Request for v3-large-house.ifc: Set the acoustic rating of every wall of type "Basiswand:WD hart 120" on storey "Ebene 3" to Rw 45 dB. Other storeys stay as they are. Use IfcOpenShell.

First a look at what the model holds.

```python
import ifcopenshell
import ifcopenshell.util.element

model = ifcopenshell.open("v3-large-house.ifc")
print(model.schema)
storey = next(s for s in model.by_type("IfcBuildingStorey") if s.Name == "Ebene 3")
walls = [e for e in ifcopenshell.util.element.get_decomposition(storey) if e.is_a("IfcWall")]
seen = {}
for e in walls:
    element_type = ifcopenshell.util.element.get_type(e)
    key = (element_type.Name if element_type != e and element_type else None, ifcopenshell.util.element.get_pset(e, "Pset_WallCommon", "AcousticRating"))
    seen[key] = seen.get(key, 0) + 1
for (name, value), count in sorted(seen.items(), key=str):
    print(count, "x", name, "|", value)
```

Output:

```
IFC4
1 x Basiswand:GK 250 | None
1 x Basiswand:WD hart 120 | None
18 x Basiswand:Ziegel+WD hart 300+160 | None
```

```python
import ifcopenshell
import ifcopenshell.api.pset
import ifcopenshell.util.element

model = ifcopenshell.open("v3-large-house.ifc")

storey = next(s for s in model.by_type("IfcBuildingStorey") if s.Name == "Ebene 3")
walls = [e for e in ifcopenshell.util.element.get_decomposition(storey) if e.is_a("IfcWall")]

count = 0
for e in walls:
    element_type = ifcopenshell.util.element.get_type(e)
    if element_type in (None, e) or element_type.Name != "Basiswand:WD hart 120":
        continue
    # add_pset returns the element's existing set when there is one.
    pset = ifcopenshell.api.pset.add_pset(model, product=e, name="Pset_WallCommon")
    ifcopenshell.api.pset.edit_pset(model, pset=pset, properties={"AcousticRating": "Rw 45 dB"})
    count += 1

print(count, "walls updated")

model.write("v3-large-house_rev.ifc")
```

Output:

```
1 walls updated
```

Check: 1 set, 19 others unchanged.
